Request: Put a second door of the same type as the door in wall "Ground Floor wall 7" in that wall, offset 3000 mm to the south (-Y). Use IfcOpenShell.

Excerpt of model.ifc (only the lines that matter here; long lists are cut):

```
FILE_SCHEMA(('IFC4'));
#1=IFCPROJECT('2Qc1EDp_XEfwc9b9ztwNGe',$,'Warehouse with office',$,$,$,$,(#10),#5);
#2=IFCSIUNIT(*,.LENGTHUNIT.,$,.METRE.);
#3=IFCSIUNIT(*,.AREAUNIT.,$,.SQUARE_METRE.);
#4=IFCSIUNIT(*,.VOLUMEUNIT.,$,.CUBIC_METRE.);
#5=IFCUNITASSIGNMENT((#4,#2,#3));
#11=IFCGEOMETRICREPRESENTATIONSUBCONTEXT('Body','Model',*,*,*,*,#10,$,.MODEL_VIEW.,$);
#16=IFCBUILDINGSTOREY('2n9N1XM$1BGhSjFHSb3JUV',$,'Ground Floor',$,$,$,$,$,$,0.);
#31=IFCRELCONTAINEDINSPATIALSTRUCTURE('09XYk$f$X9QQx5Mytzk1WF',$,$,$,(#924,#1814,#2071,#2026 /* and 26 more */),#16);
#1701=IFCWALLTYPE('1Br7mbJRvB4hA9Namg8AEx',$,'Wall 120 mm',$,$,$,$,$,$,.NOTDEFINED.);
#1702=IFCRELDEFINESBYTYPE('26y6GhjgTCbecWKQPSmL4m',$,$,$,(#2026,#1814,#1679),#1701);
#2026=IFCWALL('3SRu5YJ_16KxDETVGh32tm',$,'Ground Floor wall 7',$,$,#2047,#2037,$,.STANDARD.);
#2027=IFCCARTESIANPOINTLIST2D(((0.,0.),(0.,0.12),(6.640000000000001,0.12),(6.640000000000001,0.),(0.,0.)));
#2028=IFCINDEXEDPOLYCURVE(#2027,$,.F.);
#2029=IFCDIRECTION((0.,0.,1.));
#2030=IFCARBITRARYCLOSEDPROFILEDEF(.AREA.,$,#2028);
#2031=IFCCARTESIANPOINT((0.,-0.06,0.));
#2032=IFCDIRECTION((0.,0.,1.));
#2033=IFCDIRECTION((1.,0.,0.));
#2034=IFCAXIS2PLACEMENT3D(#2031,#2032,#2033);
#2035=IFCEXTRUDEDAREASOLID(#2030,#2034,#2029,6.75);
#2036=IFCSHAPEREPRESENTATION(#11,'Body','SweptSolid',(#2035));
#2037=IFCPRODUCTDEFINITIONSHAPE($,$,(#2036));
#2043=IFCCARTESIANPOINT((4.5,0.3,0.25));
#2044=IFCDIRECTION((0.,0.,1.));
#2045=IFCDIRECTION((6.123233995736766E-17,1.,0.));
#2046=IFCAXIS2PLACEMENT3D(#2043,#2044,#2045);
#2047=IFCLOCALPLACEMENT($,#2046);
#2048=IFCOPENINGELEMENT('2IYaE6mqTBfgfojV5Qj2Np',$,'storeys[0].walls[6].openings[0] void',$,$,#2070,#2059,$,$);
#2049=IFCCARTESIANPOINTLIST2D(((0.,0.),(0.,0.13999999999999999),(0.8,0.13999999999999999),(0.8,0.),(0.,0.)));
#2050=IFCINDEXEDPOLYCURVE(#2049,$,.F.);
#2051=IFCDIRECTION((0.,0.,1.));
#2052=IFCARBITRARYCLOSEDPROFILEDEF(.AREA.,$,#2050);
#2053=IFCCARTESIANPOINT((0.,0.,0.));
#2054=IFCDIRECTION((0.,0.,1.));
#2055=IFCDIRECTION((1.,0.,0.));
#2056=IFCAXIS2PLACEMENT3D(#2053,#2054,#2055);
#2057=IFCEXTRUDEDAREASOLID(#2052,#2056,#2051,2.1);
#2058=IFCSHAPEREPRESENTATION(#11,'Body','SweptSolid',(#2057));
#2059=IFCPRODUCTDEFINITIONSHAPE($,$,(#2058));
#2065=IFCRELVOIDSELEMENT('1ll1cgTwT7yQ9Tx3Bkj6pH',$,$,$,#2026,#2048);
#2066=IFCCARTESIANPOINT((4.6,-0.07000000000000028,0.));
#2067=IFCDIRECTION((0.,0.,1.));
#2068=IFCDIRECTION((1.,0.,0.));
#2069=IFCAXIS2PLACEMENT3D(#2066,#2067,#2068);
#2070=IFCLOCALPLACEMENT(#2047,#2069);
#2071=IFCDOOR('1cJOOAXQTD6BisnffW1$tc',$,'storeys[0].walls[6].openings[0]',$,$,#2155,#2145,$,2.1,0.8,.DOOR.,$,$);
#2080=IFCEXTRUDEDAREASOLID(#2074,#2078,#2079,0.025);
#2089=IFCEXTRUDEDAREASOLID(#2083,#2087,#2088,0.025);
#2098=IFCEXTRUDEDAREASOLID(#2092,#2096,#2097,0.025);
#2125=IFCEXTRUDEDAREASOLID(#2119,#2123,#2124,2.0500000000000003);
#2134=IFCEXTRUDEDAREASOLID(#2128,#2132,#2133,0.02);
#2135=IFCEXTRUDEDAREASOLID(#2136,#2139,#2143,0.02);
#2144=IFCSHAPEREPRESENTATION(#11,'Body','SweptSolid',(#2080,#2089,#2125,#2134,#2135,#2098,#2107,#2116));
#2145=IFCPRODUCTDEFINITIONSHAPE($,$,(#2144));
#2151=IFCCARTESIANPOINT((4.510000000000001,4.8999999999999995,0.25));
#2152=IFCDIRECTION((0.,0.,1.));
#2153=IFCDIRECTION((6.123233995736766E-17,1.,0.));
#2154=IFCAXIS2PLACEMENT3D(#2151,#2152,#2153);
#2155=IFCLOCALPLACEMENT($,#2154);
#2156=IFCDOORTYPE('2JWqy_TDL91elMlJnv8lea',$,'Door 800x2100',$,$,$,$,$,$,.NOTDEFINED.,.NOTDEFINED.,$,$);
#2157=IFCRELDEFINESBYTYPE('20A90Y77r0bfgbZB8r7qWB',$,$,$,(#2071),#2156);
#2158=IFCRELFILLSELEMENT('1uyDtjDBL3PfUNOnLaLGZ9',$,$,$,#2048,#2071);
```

```python
import ifcopenshell
import ifcopenshell.api.feature
import ifcopenshell.api.geometry
import ifcopenshell.api.root
import ifcopenshell.geom
import ifcopenshell.util.element
import ifcopenshell.util.placement
import ifcopenshell.util.shape

model = ifcopenshell.open("model.ifc")
settings = ifcopenshell.geom.settings()


def volume(element):
    """Net volume in cubic metres, openings subtracted."""
    shape = ifcopenshell.geom.create_shape(settings, element)
    return ifcopenshell.util.shape.get_volume(shape.geometry)


door = model.by_guid("1cJOOAXQTD6BisnffW1$tc")
opening = door.FillsVoids[0].RelatingOpeningElement
wall = opening.VoidsElements[0].RelatingBuildingElement
before = volume(wall)
shift = ifcopenshell.util.placement.get_local_placement(wall.ObjectPlacement)[:3, 0] * -3.0

# copy_class copies the void relationship, type, container and properties, but no geometry.
new_opening = ifcopenshell.api.root.copy_class(model, product=opening)
new_opening.Representation = ifcopenshell.util.element.copy_deep(
    model, opening.Representation, exclude=["IfcGeometricRepresentationContext", "IfcRepresentationMap"]
)
new_door = ifcopenshell.api.root.copy_class(model, product=door)
new_door.Representation = ifcopenshell.util.element.copy_deep(
    model, door.Representation, exclude=["IfcGeometricRepresentationContext", "IfcRepresentationMap"]
)
ifcopenshell.api.feature.add_filling(model, opening=new_opening, element=new_door)

for old, new in ((opening, new_opening), (door, new_door)):
    matrix = ifcopenshell.util.placement.get_local_placement(old.ObjectPlacement)
    matrix[:3, 3] += shift
    ifcopenshell.api.geometry.edit_object_placement(model, product=new, matrix=matrix, is_si=False)

after = volume(wall)

print(f"wall volume {before:.3f} -> {after:.3f} m3")

model.write("model_edited.ifc")
```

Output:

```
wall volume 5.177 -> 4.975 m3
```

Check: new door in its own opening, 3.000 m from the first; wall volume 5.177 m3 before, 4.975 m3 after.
